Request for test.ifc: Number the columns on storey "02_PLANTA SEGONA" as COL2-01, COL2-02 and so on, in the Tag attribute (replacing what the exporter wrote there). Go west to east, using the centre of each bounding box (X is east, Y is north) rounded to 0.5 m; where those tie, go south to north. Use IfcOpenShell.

First a look at what the model holds.

```python
import ifcopenshell
import ifcopenshell.util.element
import ifcopenshell.util.placement

model = ifcopenshell.open("test.ifc")
print(model.schema)
storey = next(s for s in model.by_type("IfcBuildingStorey") if s.Name == "02_PLANTA SEGONA")
columns = [e for e in ifcopenshell.util.element.get_decomposition(storey) if e.is_a("IfcColumn")]
for e in sorted(columns, key=lambda e: e.id()):
    origin = ifcopenshell.util.placement.get_local_placement(e.ObjectPlacement)[:3, 3]
    print(e.id(), e.Tag, e.Name, origin.round(2) + 0.0, sep=" | ")
```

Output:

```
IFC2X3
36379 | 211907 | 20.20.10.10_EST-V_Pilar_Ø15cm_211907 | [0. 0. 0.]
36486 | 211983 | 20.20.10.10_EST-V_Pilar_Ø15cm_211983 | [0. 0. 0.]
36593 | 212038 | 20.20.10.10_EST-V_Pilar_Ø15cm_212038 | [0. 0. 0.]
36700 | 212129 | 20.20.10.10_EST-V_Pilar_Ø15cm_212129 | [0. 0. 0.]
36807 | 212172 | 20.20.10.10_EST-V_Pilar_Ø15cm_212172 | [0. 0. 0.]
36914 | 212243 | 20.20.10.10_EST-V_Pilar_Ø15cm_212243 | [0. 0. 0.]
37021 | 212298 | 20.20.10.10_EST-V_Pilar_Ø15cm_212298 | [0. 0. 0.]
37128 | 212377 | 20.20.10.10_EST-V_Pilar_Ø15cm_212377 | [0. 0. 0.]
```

```python
import ifcopenshell
import ifcopenshell.geom
import ifcopenshell.util.element
import ifcopenshell.util.shape

model = ifcopenshell.open("test.ifc")
settings = ifcopenshell.geom.settings()
settings.set("use-world-coords", True)


def centre(element):
    shape = ifcopenshell.geom.create_shape(settings, element)
    return ifcopenshell.util.shape.get_bbox_centroid(shape.geometry)


storey = next(s for s in model.by_type("IfcBuildingStorey") if s.Name == "02_PLANTA SEGONA")
columns = [e for e in ifcopenshell.util.element.get_decomposition(storey) if e.is_a("IfcColumn")]

# Insertion points can sit at a corner or the storey origin, so sort by the geometry (in metres).
centres = {e: centre(e) for e in columns}
columns.sort(key=lambda e: (round(centres[e][0] / 0.5), centres[e][1]))

for i, e in enumerate(columns, start=1):
    number = f"COL2-{i:02d}"
    e.Tag = number
    print(e.id(), number)

model.write("test_v2.ifc")
```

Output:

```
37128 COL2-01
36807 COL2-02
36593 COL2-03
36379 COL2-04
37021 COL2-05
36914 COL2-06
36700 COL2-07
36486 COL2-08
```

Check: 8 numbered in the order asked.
